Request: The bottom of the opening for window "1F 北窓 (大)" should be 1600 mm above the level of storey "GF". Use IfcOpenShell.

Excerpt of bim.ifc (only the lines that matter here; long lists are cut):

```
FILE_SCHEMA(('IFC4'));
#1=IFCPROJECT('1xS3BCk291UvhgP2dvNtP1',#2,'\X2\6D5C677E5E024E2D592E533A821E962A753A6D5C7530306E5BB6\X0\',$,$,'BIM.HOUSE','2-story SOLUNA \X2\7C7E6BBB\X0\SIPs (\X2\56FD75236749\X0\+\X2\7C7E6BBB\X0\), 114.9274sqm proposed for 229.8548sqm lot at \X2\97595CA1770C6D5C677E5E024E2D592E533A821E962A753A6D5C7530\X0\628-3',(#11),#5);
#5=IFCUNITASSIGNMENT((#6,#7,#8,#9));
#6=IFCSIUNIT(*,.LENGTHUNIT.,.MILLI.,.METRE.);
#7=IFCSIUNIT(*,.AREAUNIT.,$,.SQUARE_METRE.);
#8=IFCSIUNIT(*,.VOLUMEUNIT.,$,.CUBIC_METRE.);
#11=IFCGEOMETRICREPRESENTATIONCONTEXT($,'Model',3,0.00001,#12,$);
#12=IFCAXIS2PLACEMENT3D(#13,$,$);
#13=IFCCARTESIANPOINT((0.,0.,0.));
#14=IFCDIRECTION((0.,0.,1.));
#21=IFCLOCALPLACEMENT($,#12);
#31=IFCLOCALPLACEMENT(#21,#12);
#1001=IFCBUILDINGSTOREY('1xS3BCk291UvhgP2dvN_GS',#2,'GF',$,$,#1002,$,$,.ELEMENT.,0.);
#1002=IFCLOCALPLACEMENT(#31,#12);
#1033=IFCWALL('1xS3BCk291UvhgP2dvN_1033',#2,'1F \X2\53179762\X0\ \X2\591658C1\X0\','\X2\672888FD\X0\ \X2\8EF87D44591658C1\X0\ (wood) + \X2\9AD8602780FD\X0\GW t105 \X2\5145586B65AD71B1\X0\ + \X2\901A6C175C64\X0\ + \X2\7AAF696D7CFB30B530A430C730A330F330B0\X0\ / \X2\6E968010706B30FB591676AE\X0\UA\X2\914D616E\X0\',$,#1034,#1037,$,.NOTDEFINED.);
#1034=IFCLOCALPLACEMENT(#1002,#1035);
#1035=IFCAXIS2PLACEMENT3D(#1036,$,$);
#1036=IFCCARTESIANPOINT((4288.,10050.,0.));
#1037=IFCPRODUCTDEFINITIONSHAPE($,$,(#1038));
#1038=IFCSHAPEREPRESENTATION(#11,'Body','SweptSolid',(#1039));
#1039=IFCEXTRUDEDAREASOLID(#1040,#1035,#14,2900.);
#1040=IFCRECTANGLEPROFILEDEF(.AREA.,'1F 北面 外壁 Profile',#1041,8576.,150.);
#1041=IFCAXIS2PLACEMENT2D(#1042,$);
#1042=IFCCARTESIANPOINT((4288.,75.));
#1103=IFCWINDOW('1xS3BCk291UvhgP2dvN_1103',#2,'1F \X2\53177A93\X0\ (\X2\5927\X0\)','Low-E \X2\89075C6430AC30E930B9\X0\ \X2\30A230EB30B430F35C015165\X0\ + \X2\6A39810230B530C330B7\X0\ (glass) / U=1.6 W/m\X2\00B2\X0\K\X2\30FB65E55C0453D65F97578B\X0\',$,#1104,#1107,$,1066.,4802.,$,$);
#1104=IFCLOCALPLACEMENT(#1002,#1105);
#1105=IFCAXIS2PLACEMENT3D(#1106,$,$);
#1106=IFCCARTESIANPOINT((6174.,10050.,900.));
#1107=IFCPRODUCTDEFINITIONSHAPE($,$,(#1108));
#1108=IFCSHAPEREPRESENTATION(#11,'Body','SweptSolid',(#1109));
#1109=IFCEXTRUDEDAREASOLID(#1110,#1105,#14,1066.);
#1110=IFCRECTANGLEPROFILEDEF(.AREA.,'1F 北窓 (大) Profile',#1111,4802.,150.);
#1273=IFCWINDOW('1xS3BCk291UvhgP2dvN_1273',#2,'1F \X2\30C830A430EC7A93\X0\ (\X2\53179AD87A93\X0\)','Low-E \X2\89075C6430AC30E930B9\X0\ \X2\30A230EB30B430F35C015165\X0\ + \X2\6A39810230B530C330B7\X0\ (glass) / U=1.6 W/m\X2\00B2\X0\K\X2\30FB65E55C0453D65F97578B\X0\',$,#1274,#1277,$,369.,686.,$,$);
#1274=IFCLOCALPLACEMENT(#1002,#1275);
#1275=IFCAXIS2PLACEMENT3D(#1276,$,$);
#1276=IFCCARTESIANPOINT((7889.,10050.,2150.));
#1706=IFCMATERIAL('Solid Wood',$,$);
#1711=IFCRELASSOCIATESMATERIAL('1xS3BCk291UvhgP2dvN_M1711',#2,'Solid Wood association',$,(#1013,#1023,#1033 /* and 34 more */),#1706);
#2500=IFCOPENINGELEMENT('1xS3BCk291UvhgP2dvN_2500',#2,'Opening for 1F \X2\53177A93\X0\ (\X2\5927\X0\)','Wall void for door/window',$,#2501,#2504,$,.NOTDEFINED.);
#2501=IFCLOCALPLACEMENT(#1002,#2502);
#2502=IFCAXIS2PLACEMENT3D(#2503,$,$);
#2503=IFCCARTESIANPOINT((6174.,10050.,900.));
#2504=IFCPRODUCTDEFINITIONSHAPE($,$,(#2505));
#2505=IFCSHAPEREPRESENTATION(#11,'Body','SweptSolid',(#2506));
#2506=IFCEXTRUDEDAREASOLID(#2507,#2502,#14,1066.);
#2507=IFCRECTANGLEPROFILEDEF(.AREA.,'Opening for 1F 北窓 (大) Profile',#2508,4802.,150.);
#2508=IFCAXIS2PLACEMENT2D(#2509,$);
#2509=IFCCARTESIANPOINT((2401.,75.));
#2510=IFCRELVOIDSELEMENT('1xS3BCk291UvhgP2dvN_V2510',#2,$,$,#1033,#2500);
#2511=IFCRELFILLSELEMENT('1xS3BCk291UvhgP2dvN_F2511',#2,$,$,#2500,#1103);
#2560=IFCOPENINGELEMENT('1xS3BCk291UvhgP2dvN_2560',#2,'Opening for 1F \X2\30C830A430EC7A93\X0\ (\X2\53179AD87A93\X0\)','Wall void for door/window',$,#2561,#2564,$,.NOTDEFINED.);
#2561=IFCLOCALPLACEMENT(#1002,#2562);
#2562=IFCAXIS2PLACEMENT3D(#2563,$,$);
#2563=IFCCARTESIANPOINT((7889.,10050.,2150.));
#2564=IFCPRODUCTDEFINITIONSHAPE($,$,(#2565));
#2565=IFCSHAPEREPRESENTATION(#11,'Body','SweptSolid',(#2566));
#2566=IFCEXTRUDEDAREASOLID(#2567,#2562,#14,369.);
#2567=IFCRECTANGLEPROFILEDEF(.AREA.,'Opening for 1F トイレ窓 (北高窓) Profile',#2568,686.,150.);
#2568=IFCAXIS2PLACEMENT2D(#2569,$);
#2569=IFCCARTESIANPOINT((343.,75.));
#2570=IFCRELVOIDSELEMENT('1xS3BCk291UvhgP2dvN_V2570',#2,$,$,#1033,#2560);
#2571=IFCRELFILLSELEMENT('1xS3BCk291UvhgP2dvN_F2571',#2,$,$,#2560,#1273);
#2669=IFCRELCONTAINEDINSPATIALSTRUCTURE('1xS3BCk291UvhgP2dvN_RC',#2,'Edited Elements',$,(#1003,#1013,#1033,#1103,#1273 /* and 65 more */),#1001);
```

```python
import numpy as np
import ifcopenshell
import ifcopenshell.api.geometry
import ifcopenshell.geom
import ifcopenshell.util.element
import ifcopenshell.util.placement
import ifcopenshell.util.shape
import ifcopenshell.util.unit

model = ifcopenshell.open("bim.ifc")
unit_scale = ifcopenshell.util.unit.calculate_unit_scale(model)

window = model.by_id(1103)
opening = window.FillsVoids[0].RelatingOpeningElement
storey = ifcopenshell.util.element.get_container(window, ifc_class="IfcBuildingStorey")
level = ifcopenshell.util.placement.get_local_placement(storey.ObjectPlacement)[2, 3]

# The opening's origin need not be at the sill, so measure its lowest point.
shape = ifcopenshell.geom.create_shape(ifcopenshell.geom.settings(), opening)
bottom = ifcopenshell.util.shape.get_shape_bottom_elevation(shape, shape.geometry) / unit_scale
dz = level + 1600.0 - bottom

shift = np.array([0.0, 0.0, dz])
# The window is not placed relative to its opening, so move both.
for product in (opening, window):
    matrix = ifcopenshell.util.placement.get_local_placement(product.ObjectPlacement)
    matrix[:3, 3] += shift
    ifcopenshell.api.geometry.edit_object_placement(model, product=product, matrix=matrix, is_si=False)

print(f"moved by {dz * unit_scale:+.3f} m")

model.write("bim_rev.ifc")
```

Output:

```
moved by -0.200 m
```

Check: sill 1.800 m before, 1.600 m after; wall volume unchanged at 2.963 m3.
